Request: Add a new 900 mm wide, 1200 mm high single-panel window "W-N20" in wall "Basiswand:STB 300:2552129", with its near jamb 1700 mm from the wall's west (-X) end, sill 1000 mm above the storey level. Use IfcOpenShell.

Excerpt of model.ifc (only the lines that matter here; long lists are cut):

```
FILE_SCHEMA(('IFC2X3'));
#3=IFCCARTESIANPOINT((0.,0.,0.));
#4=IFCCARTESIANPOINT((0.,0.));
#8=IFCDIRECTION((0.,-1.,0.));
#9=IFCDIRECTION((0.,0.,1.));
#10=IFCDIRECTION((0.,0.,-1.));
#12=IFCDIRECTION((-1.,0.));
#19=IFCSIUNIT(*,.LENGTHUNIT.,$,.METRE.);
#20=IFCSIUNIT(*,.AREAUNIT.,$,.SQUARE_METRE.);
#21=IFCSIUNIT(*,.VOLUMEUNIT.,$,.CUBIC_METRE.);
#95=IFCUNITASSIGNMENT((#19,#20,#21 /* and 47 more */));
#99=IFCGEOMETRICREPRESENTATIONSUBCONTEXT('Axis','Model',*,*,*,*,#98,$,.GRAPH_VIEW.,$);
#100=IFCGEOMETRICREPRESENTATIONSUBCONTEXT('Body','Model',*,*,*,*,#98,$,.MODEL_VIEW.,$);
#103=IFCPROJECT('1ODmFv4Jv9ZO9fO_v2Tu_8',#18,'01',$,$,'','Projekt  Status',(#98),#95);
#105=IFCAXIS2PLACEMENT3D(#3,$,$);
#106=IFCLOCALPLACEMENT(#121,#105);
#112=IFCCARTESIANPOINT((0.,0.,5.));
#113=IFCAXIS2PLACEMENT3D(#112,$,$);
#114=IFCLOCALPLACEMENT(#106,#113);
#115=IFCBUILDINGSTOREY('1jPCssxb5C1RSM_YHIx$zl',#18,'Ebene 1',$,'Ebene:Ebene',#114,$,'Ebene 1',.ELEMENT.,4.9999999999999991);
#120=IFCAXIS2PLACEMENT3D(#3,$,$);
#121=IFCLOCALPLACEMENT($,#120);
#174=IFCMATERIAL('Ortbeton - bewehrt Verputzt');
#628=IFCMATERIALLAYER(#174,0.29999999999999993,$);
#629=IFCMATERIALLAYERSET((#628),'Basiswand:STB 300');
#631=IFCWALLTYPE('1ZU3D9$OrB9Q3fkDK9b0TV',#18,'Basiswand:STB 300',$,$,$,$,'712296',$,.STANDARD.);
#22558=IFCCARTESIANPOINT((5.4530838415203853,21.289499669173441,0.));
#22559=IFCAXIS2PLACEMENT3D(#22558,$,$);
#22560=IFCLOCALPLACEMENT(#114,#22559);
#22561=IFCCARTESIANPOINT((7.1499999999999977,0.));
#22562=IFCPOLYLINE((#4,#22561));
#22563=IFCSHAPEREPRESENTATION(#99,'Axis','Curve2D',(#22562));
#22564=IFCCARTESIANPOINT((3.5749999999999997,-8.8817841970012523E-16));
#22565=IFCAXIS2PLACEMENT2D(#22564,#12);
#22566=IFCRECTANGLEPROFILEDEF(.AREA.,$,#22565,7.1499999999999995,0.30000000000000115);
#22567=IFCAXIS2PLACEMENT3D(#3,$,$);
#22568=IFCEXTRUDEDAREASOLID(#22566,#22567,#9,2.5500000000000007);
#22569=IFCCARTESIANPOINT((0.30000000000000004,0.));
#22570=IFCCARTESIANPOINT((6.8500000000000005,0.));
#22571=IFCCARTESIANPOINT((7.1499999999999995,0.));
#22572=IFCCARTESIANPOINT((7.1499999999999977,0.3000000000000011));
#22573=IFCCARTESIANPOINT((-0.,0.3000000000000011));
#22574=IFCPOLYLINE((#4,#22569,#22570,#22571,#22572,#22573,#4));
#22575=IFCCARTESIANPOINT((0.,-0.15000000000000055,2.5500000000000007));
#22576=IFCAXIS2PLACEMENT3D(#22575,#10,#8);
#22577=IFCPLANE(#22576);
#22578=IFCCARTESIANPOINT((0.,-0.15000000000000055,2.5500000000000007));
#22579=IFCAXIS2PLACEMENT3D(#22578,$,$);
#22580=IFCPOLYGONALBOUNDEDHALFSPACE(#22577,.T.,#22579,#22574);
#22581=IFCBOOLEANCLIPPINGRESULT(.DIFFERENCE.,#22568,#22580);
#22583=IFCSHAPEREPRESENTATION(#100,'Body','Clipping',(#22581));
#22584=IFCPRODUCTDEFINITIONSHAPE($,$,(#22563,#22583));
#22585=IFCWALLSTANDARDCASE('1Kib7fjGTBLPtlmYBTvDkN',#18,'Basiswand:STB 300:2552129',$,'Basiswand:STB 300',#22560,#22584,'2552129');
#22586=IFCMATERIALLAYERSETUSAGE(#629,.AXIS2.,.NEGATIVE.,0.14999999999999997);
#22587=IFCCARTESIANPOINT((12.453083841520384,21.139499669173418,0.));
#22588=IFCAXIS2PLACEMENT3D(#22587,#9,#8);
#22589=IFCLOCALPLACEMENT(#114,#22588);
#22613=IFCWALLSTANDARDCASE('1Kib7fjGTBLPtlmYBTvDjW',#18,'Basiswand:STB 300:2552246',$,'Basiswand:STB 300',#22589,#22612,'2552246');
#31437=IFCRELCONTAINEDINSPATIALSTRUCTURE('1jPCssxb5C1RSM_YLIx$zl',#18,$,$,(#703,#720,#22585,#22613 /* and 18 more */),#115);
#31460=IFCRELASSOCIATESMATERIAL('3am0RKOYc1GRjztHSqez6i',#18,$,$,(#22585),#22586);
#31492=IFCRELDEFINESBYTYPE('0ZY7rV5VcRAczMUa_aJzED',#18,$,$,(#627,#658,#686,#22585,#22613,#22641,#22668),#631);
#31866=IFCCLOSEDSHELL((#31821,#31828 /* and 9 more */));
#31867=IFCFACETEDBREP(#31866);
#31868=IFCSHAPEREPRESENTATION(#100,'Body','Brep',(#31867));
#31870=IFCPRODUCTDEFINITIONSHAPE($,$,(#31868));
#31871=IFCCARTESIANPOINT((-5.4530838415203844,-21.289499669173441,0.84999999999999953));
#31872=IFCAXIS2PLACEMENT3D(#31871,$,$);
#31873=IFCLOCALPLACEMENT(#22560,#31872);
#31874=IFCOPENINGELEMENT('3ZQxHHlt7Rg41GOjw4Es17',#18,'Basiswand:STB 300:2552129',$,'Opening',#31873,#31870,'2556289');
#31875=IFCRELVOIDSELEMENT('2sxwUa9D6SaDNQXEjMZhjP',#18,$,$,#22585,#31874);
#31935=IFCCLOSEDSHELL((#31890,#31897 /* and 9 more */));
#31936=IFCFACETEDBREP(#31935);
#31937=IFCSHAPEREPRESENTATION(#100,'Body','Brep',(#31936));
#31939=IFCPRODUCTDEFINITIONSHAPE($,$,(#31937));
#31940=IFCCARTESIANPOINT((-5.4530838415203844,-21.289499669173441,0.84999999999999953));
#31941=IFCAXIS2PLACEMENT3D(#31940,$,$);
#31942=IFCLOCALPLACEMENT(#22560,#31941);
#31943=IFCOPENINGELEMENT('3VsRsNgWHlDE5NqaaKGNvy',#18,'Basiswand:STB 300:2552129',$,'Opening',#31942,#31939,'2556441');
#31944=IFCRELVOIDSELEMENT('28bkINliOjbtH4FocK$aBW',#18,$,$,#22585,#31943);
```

```python
import numpy as np
import ifcopenshell
import ifcopenshell.api.feature
import ifcopenshell.api.geometry
import ifcopenshell.api.root
import ifcopenshell.api.spatial
import ifcopenshell.api.type
import ifcopenshell.geom
import ifcopenshell.util.element
import ifcopenshell.util.placement
import ifcopenshell.util.representation
import ifcopenshell.util.shape
import ifcopenshell.util.unit

model = ifcopenshell.open("model.ifc")
unit_scale = ifcopenshell.util.unit.calculate_unit_scale(model)
settings = ifcopenshell.geom.settings()


def volume(element):
    """Net volume in cubic metres, openings subtracted."""
    shape = ifcopenshell.geom.create_shape(settings, element)
    return ifcopenshell.util.shape.get_volume(shape.geometry)


wall = model.by_id(22585)
storey = ifcopenshell.util.element.get_container(wall, ifc_class="IfcBuildingStorey")
context = ifcopenshell.util.representation.get_context(model, "Model", "Body", "MODEL_VIEW")
before = volume(wall)

width, height, from_end, sill = 0.9, 1.2, 1.7, 1  # metres

# The wall runs along its own X axis, and the end named is its -X end.
wall_shape = ifcopenshell.geom.create_shape(settings, wall)
x, y, z = ifcopenshell.util.shape.get_vertices(wall_shape.geometry).T
start = x.min() + from_end
face, thickness = float(y.min()), float(y.max() - y.min())
wall_matrix = ifcopenshell.util.placement.get_local_placement(wall.ObjectPlacement)
level = ifcopenshell.util.placement.get_local_placement(storey.ObjectPlacement)[2, 3]


def in_wall(x, y):
    """Placement at x, y metres in the wall's axes, at sill height."""
    matrix = wall_matrix.copy()
    matrix[:, 3] = wall_matrix @ np.array([x / unit_scale, y / unit_scale, 0.0, 1.0])
    matrix[2, 3] = level + sill / unit_scale
    return matrix


# Opening: a box that overshoots both wall faces by 50 mm.
opening = ifcopenshell.api.root.create_entity(model, ifc_class="IfcOpeningElement")
box = ifcopenshell.api.geometry.add_wall_representation(
    model, context=context, length=width, height=height, thickness=thickness + 0.1
)
ifcopenshell.api.geometry.assign_representation(model, product=opening, representation=box)
ifcopenshell.api.geometry.edit_object_placement(model, product=opening, matrix=in_wall(start, face - 0.05), is_si=False)
ifcopenshell.api.feature.add_feature(model, feature=opening, element=wall)

window = ifcopenshell.api.root.create_entity(model, ifc_class="IfcWindow", name="W-N20")
window.OverallWidth, window.OverallHeight = width / unit_scale, height / unit_scale
body = ifcopenshell.api.geometry.add_window_representation(
    model,
    context=context,
    overall_width=window.OverallWidth,
    overall_height=window.OverallHeight,
    partition_type="SINGLE_PANEL",
)
ifcopenshell.api.geometry.assign_representation(model, product=window, representation=body)
ifcopenshell.api.spatial.assign_container(model, products=[window], relating_structure=storey)
fills = ifcopenshell.api.feature.add_filling(model, opening=opening, element=window)
fills.OwnerHistory = window.OwnerHistory  # required in IFC2X3

# IFC2X3 keeps the operation on the window style.
style = ifcopenshell.api.root.create_entity(model, ifc_class="IfcWindowStyle", name="W-N20")
style.OperationType, style.ConstructionType = "SINGLE_PANEL", "NOTDEFINED"
style.ParameterTakesPrecedence = style.Sizeable = False
ifcopenshell.api.type.assign_type(model, related_objects=[window], relating_type=style)

# Centre the window in the wall's thickness.
ifcopenshell.api.geometry.edit_object_placement(model, product=window, matrix=in_wall(start, face), is_si=False)
window_shape = ifcopenshell.geom.create_shape(settings, window)
depth = ifcopenshell.util.shape.get_vertices(window_shape.geometry)[:, 1]
offset = face + thickness / 2 - (depth.min() + depth.max()) / 2
ifcopenshell.api.geometry.edit_object_placement(model, product=window, matrix=in_wall(start, offset), is_si=False)

after = volume(wall)

print(f"wall volume {before:.3f} -> {after:.3f} m3")

model.write("model_edited.ifc")
```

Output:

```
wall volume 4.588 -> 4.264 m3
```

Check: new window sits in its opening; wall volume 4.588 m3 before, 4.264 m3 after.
